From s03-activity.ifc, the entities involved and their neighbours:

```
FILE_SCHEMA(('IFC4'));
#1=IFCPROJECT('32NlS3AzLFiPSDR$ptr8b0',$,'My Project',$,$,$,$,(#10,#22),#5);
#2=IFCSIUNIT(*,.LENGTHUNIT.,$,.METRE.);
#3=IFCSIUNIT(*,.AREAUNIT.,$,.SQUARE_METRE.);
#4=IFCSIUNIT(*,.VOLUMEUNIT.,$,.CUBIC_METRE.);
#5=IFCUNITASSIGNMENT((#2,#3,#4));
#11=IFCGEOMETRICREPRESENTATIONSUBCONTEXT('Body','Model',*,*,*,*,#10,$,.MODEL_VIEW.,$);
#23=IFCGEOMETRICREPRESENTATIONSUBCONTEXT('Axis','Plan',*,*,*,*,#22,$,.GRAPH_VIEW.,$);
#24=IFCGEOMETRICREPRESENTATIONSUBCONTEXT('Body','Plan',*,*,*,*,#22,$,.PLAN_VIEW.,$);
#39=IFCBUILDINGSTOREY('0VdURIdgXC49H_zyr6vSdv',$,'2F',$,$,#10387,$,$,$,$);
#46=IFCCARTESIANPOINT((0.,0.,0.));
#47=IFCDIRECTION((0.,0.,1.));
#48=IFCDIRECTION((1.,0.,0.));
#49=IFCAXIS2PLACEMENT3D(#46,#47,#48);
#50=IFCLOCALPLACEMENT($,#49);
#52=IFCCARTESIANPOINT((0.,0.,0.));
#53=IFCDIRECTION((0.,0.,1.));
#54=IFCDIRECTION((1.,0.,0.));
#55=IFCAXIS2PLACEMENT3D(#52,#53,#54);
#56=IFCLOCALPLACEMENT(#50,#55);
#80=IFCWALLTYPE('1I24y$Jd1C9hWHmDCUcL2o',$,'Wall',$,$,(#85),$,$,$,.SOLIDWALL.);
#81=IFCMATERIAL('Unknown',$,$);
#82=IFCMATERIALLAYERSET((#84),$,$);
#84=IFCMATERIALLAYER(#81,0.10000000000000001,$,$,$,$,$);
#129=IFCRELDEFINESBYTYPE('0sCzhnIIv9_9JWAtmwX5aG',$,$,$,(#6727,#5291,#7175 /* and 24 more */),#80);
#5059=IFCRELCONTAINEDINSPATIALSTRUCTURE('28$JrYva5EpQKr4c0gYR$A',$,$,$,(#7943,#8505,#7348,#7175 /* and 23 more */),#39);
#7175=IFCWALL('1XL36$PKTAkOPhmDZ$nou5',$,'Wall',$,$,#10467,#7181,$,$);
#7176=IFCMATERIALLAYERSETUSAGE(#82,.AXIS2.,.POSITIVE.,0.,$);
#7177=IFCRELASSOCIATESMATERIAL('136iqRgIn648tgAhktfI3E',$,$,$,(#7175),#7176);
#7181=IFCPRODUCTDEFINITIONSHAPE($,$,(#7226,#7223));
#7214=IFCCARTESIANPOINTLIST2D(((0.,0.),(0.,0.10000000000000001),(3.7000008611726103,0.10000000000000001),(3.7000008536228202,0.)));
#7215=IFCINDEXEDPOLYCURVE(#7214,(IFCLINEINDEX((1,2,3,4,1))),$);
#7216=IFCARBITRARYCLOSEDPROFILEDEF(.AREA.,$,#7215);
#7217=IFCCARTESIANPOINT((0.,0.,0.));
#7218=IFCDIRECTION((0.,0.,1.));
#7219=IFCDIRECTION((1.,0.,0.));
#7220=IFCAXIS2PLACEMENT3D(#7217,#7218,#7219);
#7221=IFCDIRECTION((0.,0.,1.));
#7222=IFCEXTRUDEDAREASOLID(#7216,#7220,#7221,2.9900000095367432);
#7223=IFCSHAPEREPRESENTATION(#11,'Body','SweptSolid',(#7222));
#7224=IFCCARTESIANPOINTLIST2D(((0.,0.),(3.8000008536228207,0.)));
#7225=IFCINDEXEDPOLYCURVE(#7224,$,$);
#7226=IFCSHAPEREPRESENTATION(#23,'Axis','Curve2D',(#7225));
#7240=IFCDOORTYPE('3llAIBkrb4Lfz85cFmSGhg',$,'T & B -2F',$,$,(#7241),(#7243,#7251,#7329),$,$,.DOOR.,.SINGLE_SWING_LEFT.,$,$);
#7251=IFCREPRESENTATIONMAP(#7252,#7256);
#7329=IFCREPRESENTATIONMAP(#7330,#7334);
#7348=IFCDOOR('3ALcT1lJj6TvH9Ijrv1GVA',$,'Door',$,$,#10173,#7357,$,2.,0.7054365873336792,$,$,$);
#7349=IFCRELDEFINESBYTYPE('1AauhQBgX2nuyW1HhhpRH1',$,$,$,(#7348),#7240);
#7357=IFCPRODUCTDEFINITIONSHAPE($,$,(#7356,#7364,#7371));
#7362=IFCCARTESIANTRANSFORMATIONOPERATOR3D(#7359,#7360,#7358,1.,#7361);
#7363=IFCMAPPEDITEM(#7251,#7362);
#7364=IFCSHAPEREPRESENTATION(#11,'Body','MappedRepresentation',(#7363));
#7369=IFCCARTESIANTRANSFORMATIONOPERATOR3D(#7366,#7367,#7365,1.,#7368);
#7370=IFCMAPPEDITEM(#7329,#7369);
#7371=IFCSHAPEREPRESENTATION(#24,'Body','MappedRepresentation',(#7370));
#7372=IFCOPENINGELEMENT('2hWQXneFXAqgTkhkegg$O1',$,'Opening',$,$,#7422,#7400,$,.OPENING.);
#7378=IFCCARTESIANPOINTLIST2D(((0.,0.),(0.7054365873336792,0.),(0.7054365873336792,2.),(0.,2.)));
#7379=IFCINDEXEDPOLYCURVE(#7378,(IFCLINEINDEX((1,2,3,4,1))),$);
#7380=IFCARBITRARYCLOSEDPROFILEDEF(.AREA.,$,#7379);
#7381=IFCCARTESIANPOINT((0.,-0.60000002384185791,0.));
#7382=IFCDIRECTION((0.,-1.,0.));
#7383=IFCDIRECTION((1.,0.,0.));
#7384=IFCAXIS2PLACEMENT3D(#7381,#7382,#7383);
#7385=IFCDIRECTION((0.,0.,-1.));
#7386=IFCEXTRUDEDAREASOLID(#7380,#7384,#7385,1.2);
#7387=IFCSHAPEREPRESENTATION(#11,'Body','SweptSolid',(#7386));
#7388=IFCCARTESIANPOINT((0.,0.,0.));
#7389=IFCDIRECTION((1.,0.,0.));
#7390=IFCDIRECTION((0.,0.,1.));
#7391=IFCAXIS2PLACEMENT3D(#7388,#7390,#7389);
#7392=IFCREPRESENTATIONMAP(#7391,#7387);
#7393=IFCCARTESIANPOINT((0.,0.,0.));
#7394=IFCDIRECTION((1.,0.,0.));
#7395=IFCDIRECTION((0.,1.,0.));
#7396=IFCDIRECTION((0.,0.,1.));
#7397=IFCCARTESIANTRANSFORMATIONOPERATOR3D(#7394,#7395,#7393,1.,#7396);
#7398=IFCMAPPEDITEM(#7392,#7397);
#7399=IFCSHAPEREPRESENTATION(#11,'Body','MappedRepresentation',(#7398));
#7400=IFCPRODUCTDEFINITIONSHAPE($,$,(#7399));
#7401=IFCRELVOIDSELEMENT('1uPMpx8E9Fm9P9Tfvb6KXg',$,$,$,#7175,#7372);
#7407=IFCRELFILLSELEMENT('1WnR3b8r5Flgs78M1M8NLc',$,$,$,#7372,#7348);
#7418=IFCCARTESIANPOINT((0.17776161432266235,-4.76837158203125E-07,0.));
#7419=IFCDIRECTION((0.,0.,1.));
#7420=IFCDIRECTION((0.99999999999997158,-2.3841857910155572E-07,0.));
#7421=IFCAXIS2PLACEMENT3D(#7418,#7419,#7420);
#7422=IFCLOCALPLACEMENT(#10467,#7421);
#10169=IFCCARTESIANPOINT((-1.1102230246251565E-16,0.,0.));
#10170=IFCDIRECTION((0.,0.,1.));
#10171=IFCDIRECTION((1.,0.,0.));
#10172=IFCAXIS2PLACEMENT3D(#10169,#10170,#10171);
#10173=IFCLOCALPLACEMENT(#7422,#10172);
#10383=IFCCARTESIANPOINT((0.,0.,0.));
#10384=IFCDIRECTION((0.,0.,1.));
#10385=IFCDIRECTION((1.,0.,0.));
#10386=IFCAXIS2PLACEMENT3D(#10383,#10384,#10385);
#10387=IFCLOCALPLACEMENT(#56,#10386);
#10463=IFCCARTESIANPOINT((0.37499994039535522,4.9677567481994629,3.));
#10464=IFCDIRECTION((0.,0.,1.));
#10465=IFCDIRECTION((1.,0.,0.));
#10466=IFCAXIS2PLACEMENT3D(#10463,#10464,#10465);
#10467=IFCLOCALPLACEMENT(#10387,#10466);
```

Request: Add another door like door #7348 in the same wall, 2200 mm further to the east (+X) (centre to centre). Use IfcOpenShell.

```python
import ifcopenshell
import ifcopenshell.api.feature
import ifcopenshell.api.geometry
import ifcopenshell.api.root
import ifcopenshell.geom
import ifcopenshell.util.element
import ifcopenshell.util.placement
import ifcopenshell.util.shape

model = ifcopenshell.open("s03-activity.ifc")
settings = ifcopenshell.geom.settings()


def volume(element):
    """Net volume in cubic metres, openings subtracted."""
    shape = ifcopenshell.geom.create_shape(settings, element)
    return ifcopenshell.util.shape.get_volume(shape.geometry)


door = model.by_id(7348)
opening = door.FillsVoids[0].RelatingOpeningElement
wall = opening.VoidsElements[0].RelatingBuildingElement
before = volume(wall)
shift = ifcopenshell.util.placement.get_local_placement(wall.ObjectPlacement)[:3, 0] * 2.2

# copy_class copies the void relationship, type, container and properties, but no geometry.
new_opening = ifcopenshell.api.root.copy_class(model, product=opening)
new_opening.Representation = ifcopenshell.util.element.copy_deep(
    model, opening.Representation, exclude=["IfcGeometricRepresentationContext", "IfcRepresentationMap"]
)
new_door = ifcopenshell.api.root.copy_class(model, product=door)
new_door.Representation = ifcopenshell.util.element.copy_deep(
    model, door.Representation, exclude=["IfcGeometricRepresentationContext", "IfcRepresentationMap"]
)
ifcopenshell.api.feature.add_filling(model, opening=new_opening, element=new_door)

for old, new in ((opening, new_opening), (door, new_door)):
    matrix = ifcopenshell.util.placement.get_local_placement(old.ObjectPlacement)
    matrix[:3, 3] += shift
    ifcopenshell.api.geometry.edit_object_placement(model, product=new, matrix=matrix, is_si=False)

after = volume(wall)

print(f"wall volume {before:.3f} -> {after:.3f} m3")

model.write("s03-activity_v2.ifc")
```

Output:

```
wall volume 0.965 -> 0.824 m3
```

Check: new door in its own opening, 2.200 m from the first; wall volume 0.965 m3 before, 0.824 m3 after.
